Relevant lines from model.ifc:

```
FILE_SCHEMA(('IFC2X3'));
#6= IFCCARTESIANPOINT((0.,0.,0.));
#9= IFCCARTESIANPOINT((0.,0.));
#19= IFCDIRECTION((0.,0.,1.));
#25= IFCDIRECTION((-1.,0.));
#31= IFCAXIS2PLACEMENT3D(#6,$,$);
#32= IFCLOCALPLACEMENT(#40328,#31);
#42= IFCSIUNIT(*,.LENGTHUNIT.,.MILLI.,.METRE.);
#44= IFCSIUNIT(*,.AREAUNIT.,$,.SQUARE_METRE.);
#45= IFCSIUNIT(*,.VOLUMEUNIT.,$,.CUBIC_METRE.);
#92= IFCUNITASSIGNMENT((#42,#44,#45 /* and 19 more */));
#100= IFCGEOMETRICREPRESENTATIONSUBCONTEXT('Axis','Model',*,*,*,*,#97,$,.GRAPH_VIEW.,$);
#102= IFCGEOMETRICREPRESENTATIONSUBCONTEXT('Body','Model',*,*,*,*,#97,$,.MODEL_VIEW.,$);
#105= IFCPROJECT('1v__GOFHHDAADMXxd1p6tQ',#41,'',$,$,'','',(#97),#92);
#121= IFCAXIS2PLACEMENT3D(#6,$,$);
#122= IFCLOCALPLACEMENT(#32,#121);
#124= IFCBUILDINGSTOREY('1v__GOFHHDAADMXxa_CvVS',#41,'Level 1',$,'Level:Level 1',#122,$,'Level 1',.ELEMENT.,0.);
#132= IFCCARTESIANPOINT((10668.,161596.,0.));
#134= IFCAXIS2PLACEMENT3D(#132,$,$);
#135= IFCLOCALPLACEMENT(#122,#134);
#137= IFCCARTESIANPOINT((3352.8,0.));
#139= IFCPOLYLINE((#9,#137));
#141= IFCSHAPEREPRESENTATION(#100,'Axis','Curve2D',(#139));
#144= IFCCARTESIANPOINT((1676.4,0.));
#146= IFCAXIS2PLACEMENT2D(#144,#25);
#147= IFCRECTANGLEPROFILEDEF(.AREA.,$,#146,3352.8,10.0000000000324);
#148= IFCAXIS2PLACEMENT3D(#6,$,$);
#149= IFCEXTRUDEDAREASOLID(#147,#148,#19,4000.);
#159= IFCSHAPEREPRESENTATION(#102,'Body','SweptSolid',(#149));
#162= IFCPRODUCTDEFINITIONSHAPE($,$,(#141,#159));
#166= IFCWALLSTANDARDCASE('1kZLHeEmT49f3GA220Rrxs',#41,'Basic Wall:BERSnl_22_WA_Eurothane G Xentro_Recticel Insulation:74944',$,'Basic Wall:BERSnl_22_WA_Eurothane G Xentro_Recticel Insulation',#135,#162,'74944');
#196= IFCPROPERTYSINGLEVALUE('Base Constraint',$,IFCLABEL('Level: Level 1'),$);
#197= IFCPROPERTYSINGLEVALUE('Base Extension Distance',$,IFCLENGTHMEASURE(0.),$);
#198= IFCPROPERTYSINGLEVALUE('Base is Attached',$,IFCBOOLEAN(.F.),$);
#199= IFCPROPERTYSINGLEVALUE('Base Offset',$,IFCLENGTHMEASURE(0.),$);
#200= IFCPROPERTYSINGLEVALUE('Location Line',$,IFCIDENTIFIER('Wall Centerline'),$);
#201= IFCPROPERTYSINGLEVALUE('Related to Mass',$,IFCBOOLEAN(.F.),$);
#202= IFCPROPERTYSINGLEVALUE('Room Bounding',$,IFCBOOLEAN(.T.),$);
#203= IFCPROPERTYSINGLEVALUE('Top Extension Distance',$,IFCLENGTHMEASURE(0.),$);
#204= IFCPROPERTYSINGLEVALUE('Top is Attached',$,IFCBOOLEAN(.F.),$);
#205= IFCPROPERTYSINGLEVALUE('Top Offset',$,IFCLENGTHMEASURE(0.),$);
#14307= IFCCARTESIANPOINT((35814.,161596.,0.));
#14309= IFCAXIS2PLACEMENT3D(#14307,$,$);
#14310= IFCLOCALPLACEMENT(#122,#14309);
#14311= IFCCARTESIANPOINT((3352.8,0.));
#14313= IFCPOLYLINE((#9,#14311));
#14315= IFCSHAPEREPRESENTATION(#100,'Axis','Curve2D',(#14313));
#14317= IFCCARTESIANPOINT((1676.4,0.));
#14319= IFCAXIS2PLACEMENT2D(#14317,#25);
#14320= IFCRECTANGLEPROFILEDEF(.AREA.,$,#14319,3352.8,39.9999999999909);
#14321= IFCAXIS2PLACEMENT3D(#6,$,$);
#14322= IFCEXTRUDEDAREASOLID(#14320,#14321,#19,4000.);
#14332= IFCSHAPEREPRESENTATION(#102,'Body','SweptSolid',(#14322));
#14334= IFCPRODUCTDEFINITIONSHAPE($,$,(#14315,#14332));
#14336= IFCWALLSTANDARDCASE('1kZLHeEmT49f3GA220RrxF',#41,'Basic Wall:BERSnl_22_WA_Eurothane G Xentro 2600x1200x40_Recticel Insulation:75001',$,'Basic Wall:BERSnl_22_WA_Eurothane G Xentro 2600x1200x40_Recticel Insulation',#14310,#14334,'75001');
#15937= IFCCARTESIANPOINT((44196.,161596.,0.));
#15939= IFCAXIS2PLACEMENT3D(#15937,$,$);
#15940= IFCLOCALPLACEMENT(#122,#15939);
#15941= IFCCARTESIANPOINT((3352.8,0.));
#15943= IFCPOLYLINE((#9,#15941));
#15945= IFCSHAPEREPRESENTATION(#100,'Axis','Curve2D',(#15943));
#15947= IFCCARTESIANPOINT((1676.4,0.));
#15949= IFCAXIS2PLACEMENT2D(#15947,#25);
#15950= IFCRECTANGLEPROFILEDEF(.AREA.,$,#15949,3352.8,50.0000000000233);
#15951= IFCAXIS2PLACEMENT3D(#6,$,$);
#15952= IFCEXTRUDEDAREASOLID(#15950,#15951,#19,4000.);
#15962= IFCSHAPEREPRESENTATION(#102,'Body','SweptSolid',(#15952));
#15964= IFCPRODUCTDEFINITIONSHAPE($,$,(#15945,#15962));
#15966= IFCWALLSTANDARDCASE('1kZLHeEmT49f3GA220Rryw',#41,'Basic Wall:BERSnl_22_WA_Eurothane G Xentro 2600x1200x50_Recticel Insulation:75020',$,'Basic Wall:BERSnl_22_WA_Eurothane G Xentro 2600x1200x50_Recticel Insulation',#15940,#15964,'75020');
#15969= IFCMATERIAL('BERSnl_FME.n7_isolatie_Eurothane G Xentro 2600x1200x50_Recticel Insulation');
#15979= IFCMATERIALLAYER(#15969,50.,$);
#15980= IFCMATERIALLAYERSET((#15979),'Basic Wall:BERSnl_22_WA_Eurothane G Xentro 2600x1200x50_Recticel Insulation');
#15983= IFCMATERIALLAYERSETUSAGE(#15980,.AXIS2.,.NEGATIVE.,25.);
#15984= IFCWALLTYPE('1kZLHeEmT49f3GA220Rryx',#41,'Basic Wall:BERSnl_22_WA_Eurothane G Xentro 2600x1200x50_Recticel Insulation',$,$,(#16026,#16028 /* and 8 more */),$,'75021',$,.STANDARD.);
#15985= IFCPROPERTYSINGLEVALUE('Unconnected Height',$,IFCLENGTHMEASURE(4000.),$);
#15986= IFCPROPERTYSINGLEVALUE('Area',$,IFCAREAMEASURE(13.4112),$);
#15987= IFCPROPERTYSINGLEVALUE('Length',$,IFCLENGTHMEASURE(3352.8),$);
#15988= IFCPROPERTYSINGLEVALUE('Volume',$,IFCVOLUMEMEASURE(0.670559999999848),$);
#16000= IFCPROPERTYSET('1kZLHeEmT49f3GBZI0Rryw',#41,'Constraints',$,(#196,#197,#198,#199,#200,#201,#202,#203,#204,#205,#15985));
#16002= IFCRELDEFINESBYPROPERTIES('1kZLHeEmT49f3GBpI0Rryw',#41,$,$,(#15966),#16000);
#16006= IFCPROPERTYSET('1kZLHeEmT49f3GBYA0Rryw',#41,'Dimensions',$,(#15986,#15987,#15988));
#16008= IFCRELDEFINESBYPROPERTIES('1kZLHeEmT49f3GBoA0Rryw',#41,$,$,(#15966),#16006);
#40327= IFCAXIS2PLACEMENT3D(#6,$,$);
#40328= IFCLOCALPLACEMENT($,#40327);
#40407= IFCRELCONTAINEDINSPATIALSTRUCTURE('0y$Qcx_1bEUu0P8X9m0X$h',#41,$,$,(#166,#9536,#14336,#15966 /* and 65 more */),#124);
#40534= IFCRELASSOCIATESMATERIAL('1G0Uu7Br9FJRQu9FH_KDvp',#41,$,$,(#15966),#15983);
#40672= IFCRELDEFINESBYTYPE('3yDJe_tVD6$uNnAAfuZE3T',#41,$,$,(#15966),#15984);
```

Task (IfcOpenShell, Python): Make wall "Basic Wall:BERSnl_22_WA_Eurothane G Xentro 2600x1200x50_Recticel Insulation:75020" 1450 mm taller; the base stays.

```python
import ifcopenshell
import ifcopenshell.api.pset
import ifcopenshell.geom
import ifcopenshell.util.element
import ifcopenshell.util.representation
import ifcopenshell.util.shape
import ifcopenshell.util.unit

model = ifcopenshell.open("model.ifc")
area_scale = ifcopenshell.util.unit.calculate_unit_scale(model, "AREAUNIT")
volume_scale = ifcopenshell.util.unit.calculate_unit_scale(model, "VOLUMEUNIT")
settings = ifcopenshell.geom.settings()


def volume(element):
    """Net volume in cubic metres, openings subtracted."""
    shape = ifcopenshell.geom.create_shape(settings, element)
    return ifcopenshell.util.shape.get_volume(shape.geometry)


wall = model.by_guid("1kZLHeEmT49f3GA220Rryw")
before = volume(wall)

body = ifcopenshell.util.representation.get_representation(wall, "Model", "Body")
solid = body.Items[0]
old_height = solid.Depth
solid.Depth += 1450.0
after = volume(wall)
thickness = 0.05  # wall thickness in metres

# Update the stored height, areas and volumes.
pset = model.by_id(ifcopenshell.util.element.get_pset(wall, "Constraints", should_inherit=False)["id"])
ifcopenshell.api.pset.edit_pset(model, pset=pset, properties={
    "Unconnected Height": model.create_entity("IfcLengthMeasure", solid.Depth),
})
pset = model.by_id(ifcopenshell.util.element.get_pset(wall, "Dimensions", should_inherit=False)["id"])
ifcopenshell.api.pset.edit_pset(model, pset=pset, properties={
    "Area": model.create_entity("IfcAreaMeasure", after / thickness / area_scale),
    "Volume": model.create_entity("IfcVolumeMeasure", after / volume_scale),
})

print(f"height {old_height:g} -> {solid.Depth:g}, volume {before:.3f} -> {after:.3f} m3")

model.write("model-out.ifc")
```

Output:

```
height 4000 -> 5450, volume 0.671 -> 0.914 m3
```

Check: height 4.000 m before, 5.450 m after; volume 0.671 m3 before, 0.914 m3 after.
